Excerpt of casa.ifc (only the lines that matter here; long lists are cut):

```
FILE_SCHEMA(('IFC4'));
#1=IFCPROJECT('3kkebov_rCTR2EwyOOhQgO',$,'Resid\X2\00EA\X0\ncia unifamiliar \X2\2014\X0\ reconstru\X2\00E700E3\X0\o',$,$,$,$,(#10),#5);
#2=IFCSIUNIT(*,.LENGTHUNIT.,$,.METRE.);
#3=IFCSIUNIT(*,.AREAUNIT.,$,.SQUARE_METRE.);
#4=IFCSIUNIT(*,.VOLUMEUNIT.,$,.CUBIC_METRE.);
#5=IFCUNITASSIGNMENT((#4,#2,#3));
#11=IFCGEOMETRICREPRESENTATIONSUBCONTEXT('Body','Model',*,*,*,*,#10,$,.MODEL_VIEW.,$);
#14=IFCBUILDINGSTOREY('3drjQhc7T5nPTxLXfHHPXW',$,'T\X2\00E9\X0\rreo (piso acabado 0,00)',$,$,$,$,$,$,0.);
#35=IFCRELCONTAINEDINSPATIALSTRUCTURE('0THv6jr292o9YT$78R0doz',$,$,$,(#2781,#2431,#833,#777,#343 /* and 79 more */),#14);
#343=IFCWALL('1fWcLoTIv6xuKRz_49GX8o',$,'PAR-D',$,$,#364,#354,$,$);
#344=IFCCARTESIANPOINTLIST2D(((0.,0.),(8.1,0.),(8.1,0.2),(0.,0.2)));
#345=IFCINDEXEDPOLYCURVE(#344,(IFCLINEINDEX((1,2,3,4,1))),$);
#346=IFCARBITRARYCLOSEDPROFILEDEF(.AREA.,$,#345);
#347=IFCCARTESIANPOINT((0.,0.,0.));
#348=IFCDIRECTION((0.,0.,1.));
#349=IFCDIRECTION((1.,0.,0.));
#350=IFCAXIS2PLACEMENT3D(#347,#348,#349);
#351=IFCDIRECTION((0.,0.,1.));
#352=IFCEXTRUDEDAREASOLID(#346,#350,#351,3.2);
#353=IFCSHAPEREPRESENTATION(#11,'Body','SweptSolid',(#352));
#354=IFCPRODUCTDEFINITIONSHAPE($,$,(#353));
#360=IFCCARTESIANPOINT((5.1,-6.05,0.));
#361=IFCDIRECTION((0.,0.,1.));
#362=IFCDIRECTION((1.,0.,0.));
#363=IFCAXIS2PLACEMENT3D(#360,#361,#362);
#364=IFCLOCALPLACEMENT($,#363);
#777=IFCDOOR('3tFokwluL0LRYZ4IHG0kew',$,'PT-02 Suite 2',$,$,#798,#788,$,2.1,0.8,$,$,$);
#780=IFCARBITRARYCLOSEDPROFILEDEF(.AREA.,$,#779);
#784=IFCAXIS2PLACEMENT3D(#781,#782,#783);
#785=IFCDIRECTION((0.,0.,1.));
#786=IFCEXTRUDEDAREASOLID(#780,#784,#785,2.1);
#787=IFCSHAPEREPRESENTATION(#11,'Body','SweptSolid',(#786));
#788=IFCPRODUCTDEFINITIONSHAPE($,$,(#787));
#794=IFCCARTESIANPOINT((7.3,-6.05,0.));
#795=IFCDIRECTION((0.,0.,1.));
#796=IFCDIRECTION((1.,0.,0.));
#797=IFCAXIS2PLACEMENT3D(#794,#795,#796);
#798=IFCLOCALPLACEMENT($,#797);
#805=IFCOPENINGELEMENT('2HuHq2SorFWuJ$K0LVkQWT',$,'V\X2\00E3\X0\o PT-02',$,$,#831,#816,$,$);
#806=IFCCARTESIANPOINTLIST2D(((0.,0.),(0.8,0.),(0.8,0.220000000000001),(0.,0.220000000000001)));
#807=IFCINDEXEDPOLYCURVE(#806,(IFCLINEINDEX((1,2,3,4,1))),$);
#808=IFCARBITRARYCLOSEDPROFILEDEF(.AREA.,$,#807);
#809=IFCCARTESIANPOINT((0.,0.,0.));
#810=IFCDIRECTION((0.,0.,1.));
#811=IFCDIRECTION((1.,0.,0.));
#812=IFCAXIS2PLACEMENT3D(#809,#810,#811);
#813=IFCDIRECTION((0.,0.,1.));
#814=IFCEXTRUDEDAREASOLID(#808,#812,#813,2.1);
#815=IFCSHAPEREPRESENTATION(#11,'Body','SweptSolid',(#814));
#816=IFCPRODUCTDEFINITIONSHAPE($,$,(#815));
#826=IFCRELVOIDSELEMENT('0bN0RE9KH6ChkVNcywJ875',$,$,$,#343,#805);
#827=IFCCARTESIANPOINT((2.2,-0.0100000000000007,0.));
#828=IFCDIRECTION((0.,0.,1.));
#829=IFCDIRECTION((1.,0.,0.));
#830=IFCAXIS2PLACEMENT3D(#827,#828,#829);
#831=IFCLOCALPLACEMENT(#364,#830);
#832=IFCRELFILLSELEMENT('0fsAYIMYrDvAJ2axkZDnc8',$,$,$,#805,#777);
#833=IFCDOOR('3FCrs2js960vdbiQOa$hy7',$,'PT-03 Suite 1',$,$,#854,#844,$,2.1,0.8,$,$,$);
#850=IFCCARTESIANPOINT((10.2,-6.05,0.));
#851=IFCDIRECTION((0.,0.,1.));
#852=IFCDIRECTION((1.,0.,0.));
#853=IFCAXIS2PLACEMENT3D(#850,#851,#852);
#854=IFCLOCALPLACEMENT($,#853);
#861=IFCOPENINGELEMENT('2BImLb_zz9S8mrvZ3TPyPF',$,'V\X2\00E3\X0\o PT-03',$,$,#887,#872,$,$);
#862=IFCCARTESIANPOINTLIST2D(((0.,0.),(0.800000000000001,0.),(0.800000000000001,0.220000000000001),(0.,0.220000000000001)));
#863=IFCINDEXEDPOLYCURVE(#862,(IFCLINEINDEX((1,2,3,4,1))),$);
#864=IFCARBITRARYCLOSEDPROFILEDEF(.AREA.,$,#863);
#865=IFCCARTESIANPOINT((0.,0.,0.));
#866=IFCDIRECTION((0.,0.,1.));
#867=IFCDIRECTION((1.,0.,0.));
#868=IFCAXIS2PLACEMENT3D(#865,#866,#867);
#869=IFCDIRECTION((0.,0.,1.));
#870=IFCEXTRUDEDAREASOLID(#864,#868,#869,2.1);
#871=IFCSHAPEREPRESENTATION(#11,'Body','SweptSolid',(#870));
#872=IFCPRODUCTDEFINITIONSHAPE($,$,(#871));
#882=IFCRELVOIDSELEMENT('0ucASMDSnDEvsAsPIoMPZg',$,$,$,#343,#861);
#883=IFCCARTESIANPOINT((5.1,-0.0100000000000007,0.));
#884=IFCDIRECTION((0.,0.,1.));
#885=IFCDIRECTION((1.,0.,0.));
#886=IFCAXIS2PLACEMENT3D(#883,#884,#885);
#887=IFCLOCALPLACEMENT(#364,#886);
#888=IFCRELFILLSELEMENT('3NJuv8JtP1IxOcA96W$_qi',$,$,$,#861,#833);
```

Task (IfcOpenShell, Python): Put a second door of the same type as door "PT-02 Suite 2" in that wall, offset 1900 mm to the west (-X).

```python
import ifcopenshell
import ifcopenshell.api.feature
import ifcopenshell.api.geometry
import ifcopenshell.api.root
import ifcopenshell.geom
import ifcopenshell.util.element
import ifcopenshell.util.placement
import ifcopenshell.util.shape
import ifcopenshell.util.unit

model = ifcopenshell.open("casa.ifc")
unit_scale = ifcopenshell.util.unit.calculate_unit_scale(model)
settings = ifcopenshell.geom.settings()


def volume(element):
    """Net volume in cubic metres, openings subtracted."""
    shape = ifcopenshell.geom.create_shape(settings, element)
    return ifcopenshell.util.shape.get_volume(shape.geometry)


door = model.by_guid("3tFokwluL0LRYZ4IHG0kew")
opening = door.FillsVoids[0].RelatingOpeningElement
wall = opening.VoidsElements[0].RelatingBuildingElement
before = volume(wall)
shift = ifcopenshell.util.placement.get_local_placement(wall.ObjectPlacement)[:3, 0] * -1.9 / unit_scale

# copy_class copies the void relationship, type, container and properties, but no geometry.
new_opening = ifcopenshell.api.root.copy_class(model, product=opening)
new_opening.Representation = ifcopenshell.util.element.copy_deep(
    model, opening.Representation, exclude=["IfcGeometricRepresentationContext", "IfcRepresentationMap"]
)
new_door = ifcopenshell.api.root.copy_class(model, product=door)
new_door.Representation = ifcopenshell.util.element.copy_deep(
    model, door.Representation, exclude=["IfcGeometricRepresentationContext", "IfcRepresentationMap"]
)
ifcopenshell.api.feature.add_filling(model, opening=new_opening, element=new_door)

for old, new in ((opening, new_opening), (door, new_door)):
    matrix = ifcopenshell.util.placement.get_local_placement(old.ObjectPlacement)
    matrix[:3, 3] += shift
    ifcopenshell.api.geometry.edit_object_placement(model, product=new, matrix=matrix, is_si=False)

after = volume(wall)

print(f"wall volume {before:.3f} -> {after:.3f} m3")

model.write("casa_updated.ifc")
```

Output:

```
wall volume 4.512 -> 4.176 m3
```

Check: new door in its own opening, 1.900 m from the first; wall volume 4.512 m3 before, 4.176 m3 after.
